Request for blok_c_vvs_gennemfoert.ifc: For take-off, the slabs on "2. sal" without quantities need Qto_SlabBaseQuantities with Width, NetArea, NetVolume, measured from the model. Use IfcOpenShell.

First a look at what the model holds.

```python
import ifcopenshell
import ifcopenshell.util.element
import ifcopenshell.util.unit

model = ifcopenshell.open("blok_c_vvs_gennemfoert.ifc")
print(model.schema)
for unit_type in ("LENGTHUNIT", "AREAUNIT", "VOLUMEUNIT"):
    print(unit_type, ifcopenshell.util.unit.calculate_unit_scale(model, unit_type))
storey = next(s for s in model.by_type("IfcBuildingStorey") if s.Name == "2. sal")
slabs = [e for e in ifcopenshell.util.element.get_decomposition(storey) if e.is_a("IfcSlab")]
for e in sorted(slabs, key=lambda e: e.id()):
    print(e.id(), e.is_a(), e.Name, list(ifcopenshell.util.element.get_psets(e, qtos_only=True)), sep=" | ")
```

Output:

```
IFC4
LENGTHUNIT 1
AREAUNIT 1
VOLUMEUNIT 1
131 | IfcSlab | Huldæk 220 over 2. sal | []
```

```python
import ifcopenshell
import ifcopenshell.api.pset
import ifcopenshell.geom
import ifcopenshell.util.element
import ifcopenshell.util.shape
import ifcopenshell.util.unit

model = ifcopenshell.open("blok_c_vvs_gennemfoert.ifc")
unit_scale = ifcopenshell.util.unit.calculate_unit_scale(model)
area_scale = ifcopenshell.util.unit.calculate_unit_scale(model, "AREAUNIT")
volume_scale = ifcopenshell.util.unit.calculate_unit_scale(model, "VOLUMEUNIT")
settings = ifcopenshell.geom.settings()

storey = next(s for s in model.by_type("IfcBuildingStorey") if s.Name == "2. sal")
slabs = [e for e in ifcopenshell.util.element.get_decomposition(storey) if e.is_a("IfcSlab")]

for e in sorted(slabs, key=lambda e: e.id()):
    if ifcopenshell.util.element.get_psets(e, qtos_only=True, should_inherit=False):
        continue
    # Geometry comes back in metres, in the element's own axes.
    shape = ifcopenshell.geom.create_shape(settings, e)
    values = {
        "Width": ifcopenshell.util.shape.get_z(shape.geometry) / unit_scale,
        "NetArea": ifcopenshell.util.shape.get_footprint_area(shape.geometry) / area_scale,
        "NetVolume": ifcopenshell.util.shape.get_volume(shape.geometry) / volume_scale,
    }
    qto = ifcopenshell.api.pset.add_qto(model, product=e, name="Qto_SlabBaseQuantities")
    ifcopenshell.api.pset.edit_qto(model, qto=qto, properties=values)
    print(e.id(), {k: round(v, 3) for k, v in values.items()})

model.write("blok_c_vvs_gennemfoert-out.ifc")
```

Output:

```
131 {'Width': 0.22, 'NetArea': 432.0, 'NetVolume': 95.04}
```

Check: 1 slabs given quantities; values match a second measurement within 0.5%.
